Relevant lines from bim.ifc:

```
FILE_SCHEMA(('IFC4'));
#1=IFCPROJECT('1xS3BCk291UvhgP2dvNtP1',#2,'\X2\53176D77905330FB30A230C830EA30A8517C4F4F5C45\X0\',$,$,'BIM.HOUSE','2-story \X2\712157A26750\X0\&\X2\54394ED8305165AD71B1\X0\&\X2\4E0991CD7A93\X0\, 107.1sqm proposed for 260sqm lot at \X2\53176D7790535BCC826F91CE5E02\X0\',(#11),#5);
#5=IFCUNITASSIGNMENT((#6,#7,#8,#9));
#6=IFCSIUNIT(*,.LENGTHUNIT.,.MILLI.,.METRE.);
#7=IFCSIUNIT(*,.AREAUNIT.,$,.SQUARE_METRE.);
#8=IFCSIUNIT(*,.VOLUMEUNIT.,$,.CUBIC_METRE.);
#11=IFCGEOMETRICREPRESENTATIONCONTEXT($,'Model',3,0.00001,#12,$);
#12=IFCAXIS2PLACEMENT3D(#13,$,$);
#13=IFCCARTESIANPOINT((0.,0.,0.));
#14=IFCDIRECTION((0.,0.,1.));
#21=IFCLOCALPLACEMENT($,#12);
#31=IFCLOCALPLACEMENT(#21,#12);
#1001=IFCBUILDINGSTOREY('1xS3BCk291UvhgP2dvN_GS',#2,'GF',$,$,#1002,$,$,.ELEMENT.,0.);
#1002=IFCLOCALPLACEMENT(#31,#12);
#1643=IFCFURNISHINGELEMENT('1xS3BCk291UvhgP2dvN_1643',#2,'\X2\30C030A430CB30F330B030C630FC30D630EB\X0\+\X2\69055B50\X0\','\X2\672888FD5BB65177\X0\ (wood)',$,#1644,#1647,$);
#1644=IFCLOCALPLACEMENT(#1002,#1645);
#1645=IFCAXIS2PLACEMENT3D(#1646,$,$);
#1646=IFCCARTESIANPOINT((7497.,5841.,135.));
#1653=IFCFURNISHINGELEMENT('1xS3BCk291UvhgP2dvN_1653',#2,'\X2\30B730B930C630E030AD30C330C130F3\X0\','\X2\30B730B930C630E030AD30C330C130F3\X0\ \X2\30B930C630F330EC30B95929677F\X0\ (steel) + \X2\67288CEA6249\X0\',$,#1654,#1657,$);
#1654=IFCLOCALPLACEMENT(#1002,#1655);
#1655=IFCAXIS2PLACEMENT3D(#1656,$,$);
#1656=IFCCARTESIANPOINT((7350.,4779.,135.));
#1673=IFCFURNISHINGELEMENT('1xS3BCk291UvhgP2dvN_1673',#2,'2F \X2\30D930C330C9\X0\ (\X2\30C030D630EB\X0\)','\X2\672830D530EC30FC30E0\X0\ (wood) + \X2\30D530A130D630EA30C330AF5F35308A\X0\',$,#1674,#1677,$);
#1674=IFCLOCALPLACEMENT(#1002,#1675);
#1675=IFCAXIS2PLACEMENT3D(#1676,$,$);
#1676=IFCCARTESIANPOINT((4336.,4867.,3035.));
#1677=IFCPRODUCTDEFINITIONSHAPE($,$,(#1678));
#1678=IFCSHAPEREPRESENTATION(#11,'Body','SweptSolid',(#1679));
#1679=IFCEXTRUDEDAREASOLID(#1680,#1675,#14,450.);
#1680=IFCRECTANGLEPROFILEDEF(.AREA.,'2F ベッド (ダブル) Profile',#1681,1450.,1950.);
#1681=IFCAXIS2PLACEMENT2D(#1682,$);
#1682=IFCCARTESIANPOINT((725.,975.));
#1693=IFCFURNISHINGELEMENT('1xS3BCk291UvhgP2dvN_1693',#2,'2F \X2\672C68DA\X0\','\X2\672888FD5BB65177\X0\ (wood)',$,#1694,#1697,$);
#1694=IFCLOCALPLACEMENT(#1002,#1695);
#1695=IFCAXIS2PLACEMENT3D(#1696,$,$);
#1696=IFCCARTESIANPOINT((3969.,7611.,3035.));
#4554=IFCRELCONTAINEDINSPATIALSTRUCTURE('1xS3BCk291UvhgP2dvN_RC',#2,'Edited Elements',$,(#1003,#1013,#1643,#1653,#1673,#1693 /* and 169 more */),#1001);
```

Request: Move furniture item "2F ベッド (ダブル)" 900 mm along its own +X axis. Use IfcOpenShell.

```python
import ifcopenshell
import ifcopenshell.api.geometry
import ifcopenshell.util.placement
import ifcopenshell.util.unit

model = ifcopenshell.open("bim.ifc")
unit_scale = ifcopenshell.util.unit.calculate_unit_scale(model)

item = model.by_id(1673)
matrix = ifcopenshell.util.placement.get_local_placement(item.ObjectPlacement)
matrix[:3, 3] += matrix[:3, 0] * 0.9 / unit_scale
ifcopenshell.api.geometry.edit_object_placement(model, product=item, matrix=matrix, is_si=False)

print(ifcopenshell.util.placement.get_local_placement(item.ObjectPlacement).round(3) + 0.0)

model.write("bim-out.ifc")
```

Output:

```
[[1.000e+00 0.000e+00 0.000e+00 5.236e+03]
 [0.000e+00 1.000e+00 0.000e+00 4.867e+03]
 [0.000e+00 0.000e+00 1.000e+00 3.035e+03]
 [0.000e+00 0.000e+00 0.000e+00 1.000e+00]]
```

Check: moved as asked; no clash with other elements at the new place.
